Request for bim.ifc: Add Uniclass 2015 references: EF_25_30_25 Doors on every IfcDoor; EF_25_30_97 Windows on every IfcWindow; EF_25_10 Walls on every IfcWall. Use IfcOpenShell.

First a look at what the model holds.

```python
import ifcopenshell

model = ifcopenshell.open("bim.ifc")
print(model.schema)
print("classifications:", [c.Name for c in model.by_type("IfcClassification")])
for ifc_class in ("IfcDoor", "IfcRoof", "IfcStair", "IfcWall", "IfcWindow"):
    print(ifc_class, len(model.by_type(ifc_class)))
```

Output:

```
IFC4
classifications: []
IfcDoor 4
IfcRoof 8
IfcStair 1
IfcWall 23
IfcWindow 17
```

```python
import ifcopenshell
import ifcopenshell.api.classification

model = ifcopenshell.open("bim.ifc")

system = ifcopenshell.api.classification.add_classification(model, classification="Uniclass 2015")

codes = {
    "IfcDoor": ("EF_25_30_25", "Doors"),
    "IfcWindow": ("EF_25_30_97", "Windows"),
    "IfcWall": ("EF_25_10", "Walls"),
}
for ifc_class, (code, name) in codes.items():
    products = model.by_type(ifc_class)
    ifcopenshell.api.classification.add_reference(
        model, products=products, classification=system, identification=code, name=name
    )
    print(code, len(products))

model.write("bim-out.ifc")
```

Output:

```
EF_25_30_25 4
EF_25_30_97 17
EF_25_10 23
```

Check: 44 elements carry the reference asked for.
